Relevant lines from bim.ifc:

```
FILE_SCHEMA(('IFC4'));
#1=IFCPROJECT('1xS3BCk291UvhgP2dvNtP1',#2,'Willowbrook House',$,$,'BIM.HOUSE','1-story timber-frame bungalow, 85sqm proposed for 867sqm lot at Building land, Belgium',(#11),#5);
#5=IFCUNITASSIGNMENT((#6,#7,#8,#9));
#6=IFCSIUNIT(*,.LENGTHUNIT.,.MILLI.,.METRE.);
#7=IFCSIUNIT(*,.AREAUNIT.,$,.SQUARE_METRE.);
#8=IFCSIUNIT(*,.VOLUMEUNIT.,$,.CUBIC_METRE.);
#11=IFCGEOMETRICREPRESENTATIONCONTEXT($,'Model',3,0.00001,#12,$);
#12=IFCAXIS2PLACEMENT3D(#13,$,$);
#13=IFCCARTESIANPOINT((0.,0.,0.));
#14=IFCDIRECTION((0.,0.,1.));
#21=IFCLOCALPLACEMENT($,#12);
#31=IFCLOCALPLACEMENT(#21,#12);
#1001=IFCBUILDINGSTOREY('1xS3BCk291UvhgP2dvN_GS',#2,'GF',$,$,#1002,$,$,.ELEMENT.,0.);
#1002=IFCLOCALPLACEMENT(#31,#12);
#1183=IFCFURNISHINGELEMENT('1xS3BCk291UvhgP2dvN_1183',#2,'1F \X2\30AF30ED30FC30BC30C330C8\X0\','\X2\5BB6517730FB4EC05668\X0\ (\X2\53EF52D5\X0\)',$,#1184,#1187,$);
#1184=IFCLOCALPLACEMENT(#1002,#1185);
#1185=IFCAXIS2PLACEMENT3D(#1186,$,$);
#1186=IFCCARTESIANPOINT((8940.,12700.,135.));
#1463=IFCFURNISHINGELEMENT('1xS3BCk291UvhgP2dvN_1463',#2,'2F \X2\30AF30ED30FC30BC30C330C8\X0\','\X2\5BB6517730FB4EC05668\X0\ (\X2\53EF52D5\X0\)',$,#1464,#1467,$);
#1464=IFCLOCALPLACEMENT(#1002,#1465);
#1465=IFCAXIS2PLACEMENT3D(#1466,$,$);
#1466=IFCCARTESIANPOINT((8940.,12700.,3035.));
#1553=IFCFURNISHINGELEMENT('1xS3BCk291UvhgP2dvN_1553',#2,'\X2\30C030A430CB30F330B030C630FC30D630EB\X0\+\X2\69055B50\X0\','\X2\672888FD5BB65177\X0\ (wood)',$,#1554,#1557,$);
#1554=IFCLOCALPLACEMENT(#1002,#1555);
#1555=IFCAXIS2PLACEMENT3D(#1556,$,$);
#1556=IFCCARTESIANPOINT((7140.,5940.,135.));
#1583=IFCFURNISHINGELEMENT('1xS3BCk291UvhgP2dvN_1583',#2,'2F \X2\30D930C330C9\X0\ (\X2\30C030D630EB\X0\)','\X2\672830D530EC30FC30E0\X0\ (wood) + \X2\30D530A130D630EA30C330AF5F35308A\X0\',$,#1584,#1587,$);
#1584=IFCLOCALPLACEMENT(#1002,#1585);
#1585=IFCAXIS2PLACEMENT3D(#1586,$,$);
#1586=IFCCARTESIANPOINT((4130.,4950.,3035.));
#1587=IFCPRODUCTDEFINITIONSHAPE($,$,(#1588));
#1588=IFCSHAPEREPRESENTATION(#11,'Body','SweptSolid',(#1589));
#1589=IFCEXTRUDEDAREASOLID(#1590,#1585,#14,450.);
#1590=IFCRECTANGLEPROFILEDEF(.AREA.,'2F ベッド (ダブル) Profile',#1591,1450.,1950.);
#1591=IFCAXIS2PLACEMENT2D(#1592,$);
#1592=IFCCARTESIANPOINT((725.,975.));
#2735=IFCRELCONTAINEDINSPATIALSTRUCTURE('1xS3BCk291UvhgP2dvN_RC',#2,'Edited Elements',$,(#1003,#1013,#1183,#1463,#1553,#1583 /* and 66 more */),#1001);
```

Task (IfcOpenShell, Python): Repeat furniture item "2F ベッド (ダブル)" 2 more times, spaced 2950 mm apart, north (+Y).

```python
import numpy as np
import ifcopenshell
import ifcopenshell.api.geometry
import ifcopenshell.api.root
import ifcopenshell.util.element
import ifcopenshell.util.placement

model = ifcopenshell.open("bim.ifc")


def reuse_history(source, copy):
    """copy_class also copies each property set's owner history, people and application; keep the originals."""
    for rel in copy.IsDefinedBy:
        if rel.is_a("IfcRelDefinesByProperties") and (history := rel.RelatingPropertyDefinition.OwnerHistory):
            rel.RelatingPropertyDefinition.OwnerHistory = source.OwnerHistory
            ifcopenshell.util.element.remove_deep2(model, history)


source = model.by_guid("1xS3BCk291UvhgP2dvN_1583")
base = ifcopenshell.util.placement.get_local_placement(source.ObjectPlacement)
step = np.array([0.0, 1.0, 0.0]) * 2950.0

for i in range(1, 3):
    copy = ifcopenshell.api.root.copy_class(model, product=source)
    copy.Representation = ifcopenshell.util.element.copy_deep(
        model, source.Representation, exclude=["IfcGeometricRepresentationContext", "IfcRepresentationMap"]
    )
    reuse_history(source, copy)
    matrix = base.copy()
    matrix[:3, 3] += i * step
    print("added at", matrix[:3, 3].round(3) + 0.0)
    ifcopenshell.api.geometry.edit_object_placement(model, product=copy, matrix=matrix, is_si=False)

model.write("bim_rev.ifc")
```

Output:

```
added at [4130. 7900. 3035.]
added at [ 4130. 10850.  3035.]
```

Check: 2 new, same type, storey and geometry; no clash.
